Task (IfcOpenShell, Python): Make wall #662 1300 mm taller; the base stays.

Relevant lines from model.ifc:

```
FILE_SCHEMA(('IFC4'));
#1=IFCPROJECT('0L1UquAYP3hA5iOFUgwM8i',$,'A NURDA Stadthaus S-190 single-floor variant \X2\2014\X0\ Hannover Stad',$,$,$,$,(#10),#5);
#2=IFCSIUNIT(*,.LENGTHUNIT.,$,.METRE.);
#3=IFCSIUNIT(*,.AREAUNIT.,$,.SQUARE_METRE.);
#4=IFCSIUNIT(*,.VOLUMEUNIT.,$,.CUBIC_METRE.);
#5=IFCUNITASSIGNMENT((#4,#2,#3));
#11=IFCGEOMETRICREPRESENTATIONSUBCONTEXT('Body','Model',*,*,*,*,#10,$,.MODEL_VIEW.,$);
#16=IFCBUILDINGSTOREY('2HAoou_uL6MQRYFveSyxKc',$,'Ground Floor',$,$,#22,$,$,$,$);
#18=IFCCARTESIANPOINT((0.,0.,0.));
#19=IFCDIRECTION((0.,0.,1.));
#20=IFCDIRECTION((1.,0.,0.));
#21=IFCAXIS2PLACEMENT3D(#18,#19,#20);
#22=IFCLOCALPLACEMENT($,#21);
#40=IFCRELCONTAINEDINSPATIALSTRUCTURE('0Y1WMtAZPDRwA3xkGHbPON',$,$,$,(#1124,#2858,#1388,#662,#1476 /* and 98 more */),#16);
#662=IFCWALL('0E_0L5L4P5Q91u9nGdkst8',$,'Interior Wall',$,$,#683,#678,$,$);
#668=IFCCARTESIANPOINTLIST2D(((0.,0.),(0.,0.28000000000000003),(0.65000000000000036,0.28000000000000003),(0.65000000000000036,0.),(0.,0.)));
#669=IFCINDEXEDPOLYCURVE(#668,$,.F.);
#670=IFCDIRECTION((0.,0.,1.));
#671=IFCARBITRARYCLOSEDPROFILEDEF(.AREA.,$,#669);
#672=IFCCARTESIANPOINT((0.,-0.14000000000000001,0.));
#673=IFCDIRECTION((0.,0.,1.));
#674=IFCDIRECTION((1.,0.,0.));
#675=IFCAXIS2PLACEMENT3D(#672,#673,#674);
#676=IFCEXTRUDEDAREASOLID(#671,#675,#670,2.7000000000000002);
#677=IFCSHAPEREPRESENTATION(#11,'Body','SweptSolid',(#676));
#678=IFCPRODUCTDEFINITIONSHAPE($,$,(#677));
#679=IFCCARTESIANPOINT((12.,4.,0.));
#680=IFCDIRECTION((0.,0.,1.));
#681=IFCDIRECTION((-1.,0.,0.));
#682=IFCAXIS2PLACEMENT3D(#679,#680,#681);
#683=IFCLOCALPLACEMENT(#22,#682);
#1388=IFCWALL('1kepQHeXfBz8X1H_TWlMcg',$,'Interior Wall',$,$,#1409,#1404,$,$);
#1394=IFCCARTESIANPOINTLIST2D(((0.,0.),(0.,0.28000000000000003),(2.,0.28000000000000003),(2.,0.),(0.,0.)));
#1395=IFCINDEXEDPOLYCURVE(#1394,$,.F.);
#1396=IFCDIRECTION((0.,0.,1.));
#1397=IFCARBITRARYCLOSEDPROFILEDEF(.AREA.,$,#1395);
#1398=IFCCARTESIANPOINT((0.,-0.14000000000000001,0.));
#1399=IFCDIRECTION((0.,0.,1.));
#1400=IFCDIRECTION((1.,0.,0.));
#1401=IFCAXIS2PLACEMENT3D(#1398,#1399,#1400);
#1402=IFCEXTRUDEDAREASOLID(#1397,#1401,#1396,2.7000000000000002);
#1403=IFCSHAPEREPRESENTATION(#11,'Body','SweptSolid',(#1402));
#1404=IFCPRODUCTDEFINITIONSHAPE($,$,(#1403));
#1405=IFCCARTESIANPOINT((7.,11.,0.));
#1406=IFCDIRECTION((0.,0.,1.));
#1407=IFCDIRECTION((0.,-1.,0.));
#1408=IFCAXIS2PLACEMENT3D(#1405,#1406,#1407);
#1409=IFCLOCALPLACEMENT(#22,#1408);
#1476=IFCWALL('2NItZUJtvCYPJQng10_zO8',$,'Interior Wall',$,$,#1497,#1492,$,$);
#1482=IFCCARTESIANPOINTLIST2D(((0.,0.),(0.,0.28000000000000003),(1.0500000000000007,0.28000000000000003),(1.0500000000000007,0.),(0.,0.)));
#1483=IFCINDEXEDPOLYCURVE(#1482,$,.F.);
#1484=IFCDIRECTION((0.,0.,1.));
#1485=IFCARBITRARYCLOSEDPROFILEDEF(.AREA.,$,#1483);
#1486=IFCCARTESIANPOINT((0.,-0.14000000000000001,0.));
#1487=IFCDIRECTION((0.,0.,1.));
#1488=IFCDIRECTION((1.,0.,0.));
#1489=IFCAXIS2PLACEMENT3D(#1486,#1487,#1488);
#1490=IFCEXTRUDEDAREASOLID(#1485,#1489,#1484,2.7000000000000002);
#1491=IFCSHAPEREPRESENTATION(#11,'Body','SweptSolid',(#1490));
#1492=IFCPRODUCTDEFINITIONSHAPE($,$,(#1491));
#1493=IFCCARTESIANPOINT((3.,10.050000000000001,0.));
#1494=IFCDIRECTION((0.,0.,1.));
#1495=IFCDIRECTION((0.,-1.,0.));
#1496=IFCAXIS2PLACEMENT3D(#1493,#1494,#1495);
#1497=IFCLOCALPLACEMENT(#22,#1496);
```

```python
import ifcopenshell
import ifcopenshell.geom
import ifcopenshell.util.representation
import ifcopenshell.util.shape
import ifcopenshell.util.unit

model = ifcopenshell.open("model.ifc")
unit_scale = ifcopenshell.util.unit.calculate_unit_scale(model)
settings = ifcopenshell.geom.settings()


def volume(element):
    """Net volume in cubic metres, openings subtracted."""
    shape = ifcopenshell.geom.create_shape(settings, element)
    return ifcopenshell.util.shape.get_volume(shape.geometry)


wall = model.by_guid("0E_0L5L4P5Q91u9nGdkst8")
before = volume(wall)

body = ifcopenshell.util.representation.get_representation(wall, "Model", "Body")
solid = body.Items[0]
old_height = solid.Depth
solid.Depth += 1.3 / unit_scale
after = volume(wall)

print(f"height {old_height:g} -> {solid.Depth:g}, volume {before:.3f} -> {after:.3f} m3")

model.write("model_edited.ifc")
```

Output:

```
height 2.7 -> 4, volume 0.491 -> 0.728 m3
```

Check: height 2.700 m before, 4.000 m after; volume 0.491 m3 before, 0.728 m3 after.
